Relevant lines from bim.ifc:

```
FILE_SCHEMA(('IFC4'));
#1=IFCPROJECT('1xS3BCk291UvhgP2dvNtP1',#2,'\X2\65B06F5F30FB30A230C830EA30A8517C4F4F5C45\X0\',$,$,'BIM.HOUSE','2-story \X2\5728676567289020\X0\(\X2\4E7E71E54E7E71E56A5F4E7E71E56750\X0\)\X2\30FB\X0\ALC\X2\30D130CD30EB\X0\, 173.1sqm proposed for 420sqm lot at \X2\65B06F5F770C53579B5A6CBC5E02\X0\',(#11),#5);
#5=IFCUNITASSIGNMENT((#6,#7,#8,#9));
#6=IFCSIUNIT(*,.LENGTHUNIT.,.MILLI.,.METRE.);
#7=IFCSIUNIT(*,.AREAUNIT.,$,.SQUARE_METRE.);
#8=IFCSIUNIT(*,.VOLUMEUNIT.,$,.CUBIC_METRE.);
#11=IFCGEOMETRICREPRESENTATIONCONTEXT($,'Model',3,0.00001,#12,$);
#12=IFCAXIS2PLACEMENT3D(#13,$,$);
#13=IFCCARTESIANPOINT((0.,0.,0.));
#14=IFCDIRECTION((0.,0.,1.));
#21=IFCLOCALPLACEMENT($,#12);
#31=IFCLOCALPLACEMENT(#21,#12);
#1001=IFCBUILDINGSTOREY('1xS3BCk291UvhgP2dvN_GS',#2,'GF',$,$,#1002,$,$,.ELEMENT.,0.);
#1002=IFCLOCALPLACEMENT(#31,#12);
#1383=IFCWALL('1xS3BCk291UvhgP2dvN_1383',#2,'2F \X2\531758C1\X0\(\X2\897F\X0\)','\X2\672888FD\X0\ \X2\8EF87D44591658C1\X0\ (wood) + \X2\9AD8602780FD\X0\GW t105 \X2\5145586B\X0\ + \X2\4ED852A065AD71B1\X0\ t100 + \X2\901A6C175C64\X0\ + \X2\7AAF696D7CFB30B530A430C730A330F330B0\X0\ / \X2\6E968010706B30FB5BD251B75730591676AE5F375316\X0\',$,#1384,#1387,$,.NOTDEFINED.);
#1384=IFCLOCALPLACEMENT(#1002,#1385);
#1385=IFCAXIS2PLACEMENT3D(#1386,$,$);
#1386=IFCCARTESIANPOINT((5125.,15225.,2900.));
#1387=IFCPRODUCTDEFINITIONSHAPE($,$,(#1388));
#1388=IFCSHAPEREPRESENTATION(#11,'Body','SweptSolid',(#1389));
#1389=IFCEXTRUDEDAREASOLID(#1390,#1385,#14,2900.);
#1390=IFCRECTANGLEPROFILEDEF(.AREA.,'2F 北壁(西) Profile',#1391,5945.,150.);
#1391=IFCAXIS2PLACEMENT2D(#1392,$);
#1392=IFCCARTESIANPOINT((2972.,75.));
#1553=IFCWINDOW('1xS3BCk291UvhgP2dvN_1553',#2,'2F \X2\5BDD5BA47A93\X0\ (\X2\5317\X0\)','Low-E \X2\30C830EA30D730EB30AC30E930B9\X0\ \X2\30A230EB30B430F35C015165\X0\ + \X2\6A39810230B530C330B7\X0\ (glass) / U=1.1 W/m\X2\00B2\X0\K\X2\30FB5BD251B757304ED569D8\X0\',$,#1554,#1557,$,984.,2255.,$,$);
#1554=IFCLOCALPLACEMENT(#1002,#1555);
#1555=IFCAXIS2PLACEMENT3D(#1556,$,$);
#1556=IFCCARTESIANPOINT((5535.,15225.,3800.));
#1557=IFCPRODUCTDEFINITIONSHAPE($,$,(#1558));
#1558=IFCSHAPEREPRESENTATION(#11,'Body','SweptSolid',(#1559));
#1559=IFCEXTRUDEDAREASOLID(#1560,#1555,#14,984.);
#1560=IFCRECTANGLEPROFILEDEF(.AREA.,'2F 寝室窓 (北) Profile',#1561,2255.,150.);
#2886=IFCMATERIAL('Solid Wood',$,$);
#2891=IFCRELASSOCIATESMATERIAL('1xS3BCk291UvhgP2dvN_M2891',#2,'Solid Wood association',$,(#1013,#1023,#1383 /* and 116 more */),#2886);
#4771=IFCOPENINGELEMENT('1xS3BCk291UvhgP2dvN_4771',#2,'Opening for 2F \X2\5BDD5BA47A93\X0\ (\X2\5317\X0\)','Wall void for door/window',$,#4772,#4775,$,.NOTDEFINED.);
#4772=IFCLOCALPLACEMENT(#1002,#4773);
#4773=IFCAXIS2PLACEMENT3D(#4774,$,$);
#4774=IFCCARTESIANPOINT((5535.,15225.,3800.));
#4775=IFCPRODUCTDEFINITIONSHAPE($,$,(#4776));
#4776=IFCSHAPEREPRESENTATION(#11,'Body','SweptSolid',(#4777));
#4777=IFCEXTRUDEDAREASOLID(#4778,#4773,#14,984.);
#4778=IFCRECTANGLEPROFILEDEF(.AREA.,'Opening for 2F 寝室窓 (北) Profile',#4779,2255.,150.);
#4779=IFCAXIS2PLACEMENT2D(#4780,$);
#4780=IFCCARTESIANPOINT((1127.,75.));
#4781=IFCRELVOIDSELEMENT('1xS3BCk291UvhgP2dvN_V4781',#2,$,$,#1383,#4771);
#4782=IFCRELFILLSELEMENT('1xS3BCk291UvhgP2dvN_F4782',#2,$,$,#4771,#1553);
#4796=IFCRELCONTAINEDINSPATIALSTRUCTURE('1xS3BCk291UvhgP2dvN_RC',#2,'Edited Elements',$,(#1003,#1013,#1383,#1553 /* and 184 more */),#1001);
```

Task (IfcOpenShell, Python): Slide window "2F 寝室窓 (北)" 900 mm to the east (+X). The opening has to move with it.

```python
import ifcopenshell
import ifcopenshell.api.geometry
import ifcopenshell.util.placement

model = ifcopenshell.open("bim.ifc")

window = model.by_guid("1xS3BCk291UvhgP2dvN_1553")
opening = window.FillsVoids[0].RelatingOpeningElement
wall = opening.VoidsElements[0].RelatingBuildingElement

wall_matrix = ifcopenshell.util.placement.get_local_placement(wall.ObjectPlacement)
shift = wall_matrix[:3, 0] * 900.0
before = ifcopenshell.util.placement.get_local_placement(window.ObjectPlacement)[:3, 3].copy()

# The window is not placed relative to its opening, so move both.
for product in (opening, window):
    matrix = ifcopenshell.util.placement.get_local_placement(product.ObjectPlacement)
    matrix[:3, 3] += shift
    ifcopenshell.api.geometry.edit_object_placement(model, product=product, matrix=matrix, is_si=False)

after = ifcopenshell.util.placement.get_local_placement(window.ObjectPlacement)[:3, 3]
print("window moved by", (after - before).round(3) + 0.0)

model.write("bim_updated.ifc")
```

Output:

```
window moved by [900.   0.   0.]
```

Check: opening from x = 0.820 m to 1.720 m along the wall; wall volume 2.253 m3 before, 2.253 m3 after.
